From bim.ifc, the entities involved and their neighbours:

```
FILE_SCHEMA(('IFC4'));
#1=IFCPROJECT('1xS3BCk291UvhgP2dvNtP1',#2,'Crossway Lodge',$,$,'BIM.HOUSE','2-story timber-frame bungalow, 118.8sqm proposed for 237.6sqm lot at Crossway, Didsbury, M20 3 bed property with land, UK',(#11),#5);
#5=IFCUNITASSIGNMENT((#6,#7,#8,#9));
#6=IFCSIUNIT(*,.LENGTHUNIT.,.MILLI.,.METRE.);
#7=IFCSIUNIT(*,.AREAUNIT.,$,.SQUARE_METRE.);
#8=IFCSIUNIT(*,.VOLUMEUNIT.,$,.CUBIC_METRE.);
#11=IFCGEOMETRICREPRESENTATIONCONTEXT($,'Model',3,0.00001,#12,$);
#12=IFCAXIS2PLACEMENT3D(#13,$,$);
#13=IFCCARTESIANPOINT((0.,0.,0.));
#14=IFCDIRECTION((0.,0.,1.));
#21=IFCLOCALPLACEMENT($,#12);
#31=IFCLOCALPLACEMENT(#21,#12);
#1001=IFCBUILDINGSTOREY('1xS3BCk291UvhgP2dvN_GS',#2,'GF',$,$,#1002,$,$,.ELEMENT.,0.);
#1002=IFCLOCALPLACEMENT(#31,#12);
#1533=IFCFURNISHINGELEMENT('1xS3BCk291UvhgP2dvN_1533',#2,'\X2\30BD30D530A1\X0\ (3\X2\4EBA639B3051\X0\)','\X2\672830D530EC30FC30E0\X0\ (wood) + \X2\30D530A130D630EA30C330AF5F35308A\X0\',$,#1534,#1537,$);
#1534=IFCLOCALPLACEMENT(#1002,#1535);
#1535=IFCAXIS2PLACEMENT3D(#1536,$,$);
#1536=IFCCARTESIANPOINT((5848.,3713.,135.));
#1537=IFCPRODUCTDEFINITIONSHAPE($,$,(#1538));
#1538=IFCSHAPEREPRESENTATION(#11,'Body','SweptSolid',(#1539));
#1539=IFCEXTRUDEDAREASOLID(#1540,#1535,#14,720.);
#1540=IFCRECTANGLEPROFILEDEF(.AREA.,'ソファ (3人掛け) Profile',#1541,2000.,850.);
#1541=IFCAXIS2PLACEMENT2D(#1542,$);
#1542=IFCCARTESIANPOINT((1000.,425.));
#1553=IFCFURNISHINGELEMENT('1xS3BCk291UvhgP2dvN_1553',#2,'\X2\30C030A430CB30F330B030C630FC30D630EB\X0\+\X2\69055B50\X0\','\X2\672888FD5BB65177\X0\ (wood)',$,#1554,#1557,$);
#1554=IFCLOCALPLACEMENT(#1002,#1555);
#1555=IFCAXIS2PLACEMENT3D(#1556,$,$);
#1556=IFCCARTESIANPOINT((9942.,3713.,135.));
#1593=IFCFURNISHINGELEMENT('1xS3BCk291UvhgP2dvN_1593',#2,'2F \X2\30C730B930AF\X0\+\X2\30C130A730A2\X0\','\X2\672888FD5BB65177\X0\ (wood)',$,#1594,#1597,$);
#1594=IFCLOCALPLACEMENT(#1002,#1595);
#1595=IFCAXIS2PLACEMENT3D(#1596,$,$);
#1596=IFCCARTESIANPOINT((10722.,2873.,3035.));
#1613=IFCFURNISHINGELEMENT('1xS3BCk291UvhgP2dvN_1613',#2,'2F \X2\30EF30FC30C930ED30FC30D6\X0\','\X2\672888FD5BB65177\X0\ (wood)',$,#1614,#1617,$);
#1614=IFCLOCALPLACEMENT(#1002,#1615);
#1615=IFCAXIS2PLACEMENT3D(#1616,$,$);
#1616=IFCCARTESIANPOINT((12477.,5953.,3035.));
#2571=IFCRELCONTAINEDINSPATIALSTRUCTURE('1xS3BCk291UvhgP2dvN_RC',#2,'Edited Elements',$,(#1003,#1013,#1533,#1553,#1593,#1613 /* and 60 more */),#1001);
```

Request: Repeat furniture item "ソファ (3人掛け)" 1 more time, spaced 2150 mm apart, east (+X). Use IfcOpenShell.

```python
import numpy as np
import ifcopenshell
import ifcopenshell.api.geometry
import ifcopenshell.api.root
import ifcopenshell.util.element
import ifcopenshell.util.placement

model = ifcopenshell.open("bim.ifc")


def reuse_history(source, copy):
    """copy_class also copies each property set's owner history, people and application; keep the originals."""
    for rel in copy.IsDefinedBy:
        if rel.is_a("IfcRelDefinesByProperties") and (history := rel.RelatingPropertyDefinition.OwnerHistory):
            rel.RelatingPropertyDefinition.OwnerHistory = source.OwnerHistory
            ifcopenshell.util.element.remove_deep2(model, history)


source = model.by_guid("1xS3BCk291UvhgP2dvN_1533")
base = ifcopenshell.util.placement.get_local_placement(source.ObjectPlacement)
step = np.array([1.0, 0.0, 0.0]) * 2150.0

for i in range(1, 2):
    copy = ifcopenshell.api.root.copy_class(model, product=source)
    copy.Representation = ifcopenshell.util.element.copy_deep(
        model, source.Representation, exclude=["IfcGeometricRepresentationContext", "IfcRepresentationMap"]
    )
    reuse_history(source, copy)
    matrix = base.copy()
    matrix[:3, 3] += i * step
    print("added at", matrix[:3, 3].round(3) + 0.0)
    ifcopenshell.api.geometry.edit_object_placement(model, product=copy, matrix=matrix, is_si=False)

model.write("bim-out.ifc")
```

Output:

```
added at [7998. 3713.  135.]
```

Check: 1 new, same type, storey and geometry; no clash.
